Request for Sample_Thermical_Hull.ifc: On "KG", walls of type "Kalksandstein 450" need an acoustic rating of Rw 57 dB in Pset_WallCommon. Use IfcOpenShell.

First a look at what the model holds.

```python
import ifcopenshell
import ifcopenshell.util.element

model = ifcopenshell.open("Sample_Thermical_Hull.ifc")
print(model.schema)
storey = next(s for s in model.by_type("IfcBuildingStorey") if s.Name == "KG")
walls = [e for e in ifcopenshell.util.element.get_decomposition(storey) if e.is_a("IfcWall")]
seen = {}
for e in walls:
    element_type = ifcopenshell.util.element.get_type(e)
    key = (element_type.Name if element_type != e and element_type else None, ifcopenshell.util.element.get_pset(e, "Pset_WallCommon", "AcousticRating"))
    seen[key] = seen.get(key, 0) + 1
for (name, value), count in sorted(seen.items(), key=str):
    print(count, "x", name, "|", value)
```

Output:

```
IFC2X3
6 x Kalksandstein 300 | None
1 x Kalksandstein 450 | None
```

```python
import ifcopenshell
import ifcopenshell.api.pset
import ifcopenshell.util.element

model = ifcopenshell.open("Sample_Thermical_Hull.ifc")

storey = next(s for s in model.by_type("IfcBuildingStorey") if s.Name == "KG")
walls = [e for e in ifcopenshell.util.element.get_decomposition(storey) if e.is_a("IfcWall")]

count = 0
for e in walls:
    element_type = ifcopenshell.util.element.get_type(e)
    if element_type in (None, e) or element_type.Name != "Kalksandstein 450":
        continue
    # add_pset returns the element's existing set when there is one.
    pset = ifcopenshell.api.pset.add_pset(model, product=e, name="Pset_WallCommon")
    ifcopenshell.api.pset.edit_pset(model, pset=pset, properties={"AcousticRating": "Rw 57 dB"})
    count += 1

print(count, "walls updated")

model.write("Sample_Thermical_Hull-out.ifc")
```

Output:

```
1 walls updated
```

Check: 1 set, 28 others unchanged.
